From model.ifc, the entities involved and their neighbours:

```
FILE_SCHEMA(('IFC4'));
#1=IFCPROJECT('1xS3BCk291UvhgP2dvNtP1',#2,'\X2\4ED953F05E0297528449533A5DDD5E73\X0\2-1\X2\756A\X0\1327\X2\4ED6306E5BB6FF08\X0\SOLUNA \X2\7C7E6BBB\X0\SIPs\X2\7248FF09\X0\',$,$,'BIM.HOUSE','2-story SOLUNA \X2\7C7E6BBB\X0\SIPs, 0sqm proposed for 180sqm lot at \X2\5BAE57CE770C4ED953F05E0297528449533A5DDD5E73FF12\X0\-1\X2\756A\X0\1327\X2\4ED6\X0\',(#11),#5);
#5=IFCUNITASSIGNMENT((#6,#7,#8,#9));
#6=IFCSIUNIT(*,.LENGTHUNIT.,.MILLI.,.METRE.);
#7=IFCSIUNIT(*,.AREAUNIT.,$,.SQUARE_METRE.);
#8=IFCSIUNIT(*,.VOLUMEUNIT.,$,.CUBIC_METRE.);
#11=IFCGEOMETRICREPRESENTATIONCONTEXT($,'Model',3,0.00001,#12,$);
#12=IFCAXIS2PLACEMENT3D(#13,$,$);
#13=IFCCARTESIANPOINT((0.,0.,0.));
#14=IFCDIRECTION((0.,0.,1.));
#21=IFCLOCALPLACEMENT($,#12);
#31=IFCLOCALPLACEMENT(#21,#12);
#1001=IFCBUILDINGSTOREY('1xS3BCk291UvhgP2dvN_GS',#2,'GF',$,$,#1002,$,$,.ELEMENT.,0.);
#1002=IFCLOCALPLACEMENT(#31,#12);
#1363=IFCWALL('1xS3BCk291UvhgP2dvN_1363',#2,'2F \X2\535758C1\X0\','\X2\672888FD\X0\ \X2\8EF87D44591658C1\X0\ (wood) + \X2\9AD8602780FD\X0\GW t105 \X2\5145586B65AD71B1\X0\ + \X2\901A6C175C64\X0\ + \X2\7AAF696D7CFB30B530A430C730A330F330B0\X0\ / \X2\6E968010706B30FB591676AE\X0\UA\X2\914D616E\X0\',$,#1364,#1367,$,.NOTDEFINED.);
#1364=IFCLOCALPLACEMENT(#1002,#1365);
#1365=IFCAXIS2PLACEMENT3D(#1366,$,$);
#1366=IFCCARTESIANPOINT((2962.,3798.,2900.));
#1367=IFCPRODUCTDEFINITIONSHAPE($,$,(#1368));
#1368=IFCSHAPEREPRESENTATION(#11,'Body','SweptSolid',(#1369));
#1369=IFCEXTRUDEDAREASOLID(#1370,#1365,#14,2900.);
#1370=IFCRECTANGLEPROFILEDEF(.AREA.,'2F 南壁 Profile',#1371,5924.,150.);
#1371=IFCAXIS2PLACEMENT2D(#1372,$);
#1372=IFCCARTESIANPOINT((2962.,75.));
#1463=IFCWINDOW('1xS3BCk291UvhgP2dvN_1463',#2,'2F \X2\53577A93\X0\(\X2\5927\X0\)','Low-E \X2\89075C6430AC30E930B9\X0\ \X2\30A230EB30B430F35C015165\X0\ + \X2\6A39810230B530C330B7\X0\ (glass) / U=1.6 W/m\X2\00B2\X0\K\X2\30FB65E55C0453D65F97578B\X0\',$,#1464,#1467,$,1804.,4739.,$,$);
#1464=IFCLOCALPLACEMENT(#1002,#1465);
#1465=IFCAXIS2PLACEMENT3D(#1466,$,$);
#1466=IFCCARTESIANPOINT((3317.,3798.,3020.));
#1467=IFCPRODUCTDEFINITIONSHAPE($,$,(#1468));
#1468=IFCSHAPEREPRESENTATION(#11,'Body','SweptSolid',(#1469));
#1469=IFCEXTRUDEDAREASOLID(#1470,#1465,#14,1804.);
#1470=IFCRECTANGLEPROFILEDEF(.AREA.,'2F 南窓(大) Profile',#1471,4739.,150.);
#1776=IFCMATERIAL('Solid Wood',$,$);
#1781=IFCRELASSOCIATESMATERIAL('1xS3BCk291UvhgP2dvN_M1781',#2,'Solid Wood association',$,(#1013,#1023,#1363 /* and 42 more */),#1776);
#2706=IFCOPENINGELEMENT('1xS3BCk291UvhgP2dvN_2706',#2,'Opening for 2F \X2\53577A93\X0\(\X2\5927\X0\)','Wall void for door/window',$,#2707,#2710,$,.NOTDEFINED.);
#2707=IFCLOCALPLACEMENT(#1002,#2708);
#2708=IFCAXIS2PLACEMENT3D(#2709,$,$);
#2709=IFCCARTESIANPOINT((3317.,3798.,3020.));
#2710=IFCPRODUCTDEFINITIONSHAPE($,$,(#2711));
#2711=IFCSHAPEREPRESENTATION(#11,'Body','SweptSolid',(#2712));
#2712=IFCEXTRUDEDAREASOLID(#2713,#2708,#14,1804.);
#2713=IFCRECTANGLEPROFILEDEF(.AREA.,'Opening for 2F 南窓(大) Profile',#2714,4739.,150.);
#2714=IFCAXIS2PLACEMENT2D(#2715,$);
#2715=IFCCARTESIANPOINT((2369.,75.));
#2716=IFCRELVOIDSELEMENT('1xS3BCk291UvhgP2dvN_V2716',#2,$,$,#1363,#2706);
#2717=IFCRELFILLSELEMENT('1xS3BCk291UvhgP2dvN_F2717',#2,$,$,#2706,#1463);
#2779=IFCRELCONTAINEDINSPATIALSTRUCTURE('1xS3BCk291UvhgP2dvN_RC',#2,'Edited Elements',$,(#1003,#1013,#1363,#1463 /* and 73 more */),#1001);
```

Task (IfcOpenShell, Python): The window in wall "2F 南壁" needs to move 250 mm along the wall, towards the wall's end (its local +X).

```python
import ifcopenshell
import ifcopenshell.api.geometry
import ifcopenshell.util.placement
import ifcopenshell.util.unit

model = ifcopenshell.open("model.ifc")
unit_scale = ifcopenshell.util.unit.calculate_unit_scale(model)

window = model.by_guid("1xS3BCk291UvhgP2dvN_1463")
opening = window.FillsVoids[0].RelatingOpeningElement
wall = opening.VoidsElements[0].RelatingBuildingElement

wall_matrix = ifcopenshell.util.placement.get_local_placement(wall.ObjectPlacement)
shift = wall_matrix[:3, 0] * 0.25 / unit_scale
before = ifcopenshell.util.placement.get_local_placement(window.ObjectPlacement)[:3, 3].copy()

# The window is not placed relative to its opening, so move both.
for product in (opening, window):
    matrix = ifcopenshell.util.placement.get_local_placement(product.ObjectPlacement)
    matrix[:3, 3] += shift
    ifcopenshell.api.geometry.edit_object_placement(model, product=product, matrix=matrix, is_si=False)

after = ifcopenshell.util.placement.get_local_placement(window.ObjectPlacement)[:3, 3]
print("window moved by", (after - before).round(3) + 0.0)

model.write("model_v2.ifc")
```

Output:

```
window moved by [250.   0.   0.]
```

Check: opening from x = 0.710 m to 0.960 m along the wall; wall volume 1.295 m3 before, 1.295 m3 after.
